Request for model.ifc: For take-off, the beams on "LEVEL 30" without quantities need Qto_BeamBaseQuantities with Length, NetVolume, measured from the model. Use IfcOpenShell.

First a look at what the model holds.

```python
import ifcopenshell
import ifcopenshell.util.element
import ifcopenshell.util.unit

model = ifcopenshell.open("model.ifc")
print(model.schema)
for unit_type in ("LENGTHUNIT", "AREAUNIT", "VOLUMEUNIT"):
    print(unit_type, ifcopenshell.util.unit.calculate_unit_scale(model, unit_type))
storey = next(s for s in model.by_type("IfcBuildingStorey") if s.Name == "LEVEL 30")
beams = [e for e in ifcopenshell.util.element.get_decomposition(storey) if e.is_a("IfcBeam")]
for e in sorted(beams, key=lambda e: e.id()):
    print(e.id(), e.is_a(), e.Name, list(ifcopenshell.util.element.get_psets(e, qtos_only=True)), sep=" | ")
```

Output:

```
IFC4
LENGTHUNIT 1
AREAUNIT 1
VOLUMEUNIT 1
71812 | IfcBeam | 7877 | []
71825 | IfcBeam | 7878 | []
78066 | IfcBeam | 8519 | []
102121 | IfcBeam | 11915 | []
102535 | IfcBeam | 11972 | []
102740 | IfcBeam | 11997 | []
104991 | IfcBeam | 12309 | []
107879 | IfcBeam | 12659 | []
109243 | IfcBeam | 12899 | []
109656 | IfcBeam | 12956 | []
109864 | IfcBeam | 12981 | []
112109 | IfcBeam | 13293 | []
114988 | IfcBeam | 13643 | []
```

```python
import ifcopenshell
import ifcopenshell.api.pset
import ifcopenshell.geom
import ifcopenshell.util.element
import ifcopenshell.util.shape
import ifcopenshell.util.unit

model = ifcopenshell.open("model.ifc")
unit_scale = ifcopenshell.util.unit.calculate_unit_scale(model)
volume_scale = ifcopenshell.util.unit.calculate_unit_scale(model, "VOLUMEUNIT")
settings = ifcopenshell.geom.settings()

storey = next(s for s in model.by_type("IfcBuildingStorey") if s.Name == "LEVEL 30")
beams = [e for e in ifcopenshell.util.element.get_decomposition(storey) if e.is_a("IfcBeam")]

for e in sorted(beams, key=lambda e: e.id()):
    if ifcopenshell.util.element.get_psets(e, qtos_only=True, should_inherit=False):
        continue
    # Geometry comes back in metres, in the element's own axes.
    shape = ifcopenshell.geom.create_shape(settings, e)
    values = {
        "Length": ifcopenshell.util.shape.get_max_xyz(shape.geometry) / unit_scale,
        "NetVolume": ifcopenshell.util.shape.get_volume(shape.geometry) / volume_scale,
    }
    qto = ifcopenshell.api.pset.add_qto(model, product=e, name="Qto_BeamBaseQuantities")
    ifcopenshell.api.pset.edit_qto(model, qto=qto, properties=values)
    print(e.id(), {k: round(v, 3) for k, v in values.items()})

model.write("model_edited.ifc")
```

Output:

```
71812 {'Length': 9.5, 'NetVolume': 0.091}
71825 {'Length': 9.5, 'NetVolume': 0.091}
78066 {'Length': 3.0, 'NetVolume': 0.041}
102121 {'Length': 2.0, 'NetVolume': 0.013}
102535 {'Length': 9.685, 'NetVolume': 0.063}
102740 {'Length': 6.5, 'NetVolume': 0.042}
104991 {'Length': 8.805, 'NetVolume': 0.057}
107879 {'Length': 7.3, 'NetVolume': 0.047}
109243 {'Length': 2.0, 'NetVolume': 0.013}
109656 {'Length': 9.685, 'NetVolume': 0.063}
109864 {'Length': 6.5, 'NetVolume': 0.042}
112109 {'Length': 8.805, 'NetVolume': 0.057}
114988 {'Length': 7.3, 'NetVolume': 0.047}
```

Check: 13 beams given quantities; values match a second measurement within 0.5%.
